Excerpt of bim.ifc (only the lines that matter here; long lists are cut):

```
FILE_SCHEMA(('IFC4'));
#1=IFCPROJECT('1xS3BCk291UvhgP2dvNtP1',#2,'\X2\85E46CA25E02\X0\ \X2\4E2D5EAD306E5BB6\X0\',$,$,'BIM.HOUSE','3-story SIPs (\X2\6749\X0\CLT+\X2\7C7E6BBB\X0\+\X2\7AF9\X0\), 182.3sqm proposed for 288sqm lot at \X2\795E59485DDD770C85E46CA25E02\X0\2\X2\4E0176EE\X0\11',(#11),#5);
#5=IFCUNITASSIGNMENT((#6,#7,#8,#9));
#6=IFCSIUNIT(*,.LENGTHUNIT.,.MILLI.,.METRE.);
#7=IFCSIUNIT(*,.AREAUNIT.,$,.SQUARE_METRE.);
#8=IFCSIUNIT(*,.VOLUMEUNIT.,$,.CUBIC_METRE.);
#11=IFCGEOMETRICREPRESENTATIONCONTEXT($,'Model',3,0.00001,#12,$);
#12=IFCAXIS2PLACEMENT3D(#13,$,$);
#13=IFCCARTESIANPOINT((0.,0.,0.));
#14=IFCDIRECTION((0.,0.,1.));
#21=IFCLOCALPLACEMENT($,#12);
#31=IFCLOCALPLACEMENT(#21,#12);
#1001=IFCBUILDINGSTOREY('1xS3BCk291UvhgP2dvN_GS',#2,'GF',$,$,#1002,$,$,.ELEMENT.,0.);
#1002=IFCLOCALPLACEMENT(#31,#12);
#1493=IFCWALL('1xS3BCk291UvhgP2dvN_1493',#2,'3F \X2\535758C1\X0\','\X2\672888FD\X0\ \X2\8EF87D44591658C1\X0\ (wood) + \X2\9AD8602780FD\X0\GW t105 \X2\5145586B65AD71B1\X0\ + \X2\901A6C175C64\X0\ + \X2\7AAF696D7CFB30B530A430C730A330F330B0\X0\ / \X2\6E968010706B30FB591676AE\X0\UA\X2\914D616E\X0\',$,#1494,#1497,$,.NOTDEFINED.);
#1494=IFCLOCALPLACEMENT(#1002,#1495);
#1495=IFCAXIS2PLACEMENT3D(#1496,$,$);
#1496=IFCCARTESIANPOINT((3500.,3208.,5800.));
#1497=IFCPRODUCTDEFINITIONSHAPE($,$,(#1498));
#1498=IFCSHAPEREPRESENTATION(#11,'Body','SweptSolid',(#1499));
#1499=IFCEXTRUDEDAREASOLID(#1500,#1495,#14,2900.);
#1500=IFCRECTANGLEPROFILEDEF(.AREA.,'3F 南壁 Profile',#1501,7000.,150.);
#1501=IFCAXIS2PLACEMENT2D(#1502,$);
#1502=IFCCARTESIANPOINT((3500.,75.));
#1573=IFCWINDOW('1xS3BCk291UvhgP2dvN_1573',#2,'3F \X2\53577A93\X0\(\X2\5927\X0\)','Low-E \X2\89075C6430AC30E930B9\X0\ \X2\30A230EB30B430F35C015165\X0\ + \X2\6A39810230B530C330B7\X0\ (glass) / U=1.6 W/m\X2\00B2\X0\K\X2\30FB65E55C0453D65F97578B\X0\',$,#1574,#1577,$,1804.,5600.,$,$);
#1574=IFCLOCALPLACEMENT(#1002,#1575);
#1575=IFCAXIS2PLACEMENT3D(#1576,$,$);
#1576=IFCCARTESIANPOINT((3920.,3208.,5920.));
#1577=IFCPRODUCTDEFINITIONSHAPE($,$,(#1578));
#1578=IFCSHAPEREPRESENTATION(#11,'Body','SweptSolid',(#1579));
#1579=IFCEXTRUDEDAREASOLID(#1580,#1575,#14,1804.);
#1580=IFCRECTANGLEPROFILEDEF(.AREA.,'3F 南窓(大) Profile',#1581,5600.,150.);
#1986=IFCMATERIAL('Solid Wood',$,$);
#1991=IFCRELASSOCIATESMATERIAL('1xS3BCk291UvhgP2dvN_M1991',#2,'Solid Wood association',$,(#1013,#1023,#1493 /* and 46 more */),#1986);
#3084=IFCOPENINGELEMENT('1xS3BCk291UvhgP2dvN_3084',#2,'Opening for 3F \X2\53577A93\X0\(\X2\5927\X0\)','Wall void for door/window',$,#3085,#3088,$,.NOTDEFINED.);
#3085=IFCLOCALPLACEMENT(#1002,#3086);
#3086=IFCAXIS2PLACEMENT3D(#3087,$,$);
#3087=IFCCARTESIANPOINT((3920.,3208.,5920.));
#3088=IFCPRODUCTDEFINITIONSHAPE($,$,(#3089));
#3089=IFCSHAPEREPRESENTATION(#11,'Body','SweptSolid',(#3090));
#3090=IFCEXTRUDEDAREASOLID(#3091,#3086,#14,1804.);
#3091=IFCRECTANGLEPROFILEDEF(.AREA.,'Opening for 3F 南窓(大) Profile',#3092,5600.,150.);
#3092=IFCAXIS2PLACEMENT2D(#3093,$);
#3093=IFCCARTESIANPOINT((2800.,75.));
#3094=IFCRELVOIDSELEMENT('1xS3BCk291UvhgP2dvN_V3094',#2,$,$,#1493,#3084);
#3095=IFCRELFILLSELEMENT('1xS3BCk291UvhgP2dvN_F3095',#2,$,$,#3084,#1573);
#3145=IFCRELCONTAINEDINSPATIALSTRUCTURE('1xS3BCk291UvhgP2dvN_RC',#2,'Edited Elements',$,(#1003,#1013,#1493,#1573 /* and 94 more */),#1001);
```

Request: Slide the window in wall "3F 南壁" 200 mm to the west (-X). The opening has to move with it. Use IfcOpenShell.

```python
import ifcopenshell
import ifcopenshell.api.geometry
import ifcopenshell.util.placement

model = ifcopenshell.open("bim.ifc")

window = model.by_guid("1xS3BCk291UvhgP2dvN_1573")
opening = window.FillsVoids[0].RelatingOpeningElement
wall = opening.VoidsElements[0].RelatingBuildingElement

wall_matrix = ifcopenshell.util.placement.get_local_placement(wall.ObjectPlacement)
shift = wall_matrix[:3, 0] * -200.0
before = ifcopenshell.util.placement.get_local_placement(window.ObjectPlacement)[:3, 3].copy()

# The window is not placed relative to its opening, so move both.
for product in (opening, window):
    matrix = ifcopenshell.util.placement.get_local_placement(product.ObjectPlacement)
    matrix[:3, 3] += shift
    ifcopenshell.api.geometry.edit_object_placement(model, product=product, matrix=matrix, is_si=False)

after = ifcopenshell.util.placement.get_local_placement(window.ObjectPlacement)[:3, 3]
print("window moved by", (after - before).round(3) + 0.0)

model.write("bim_edited.ifc")
```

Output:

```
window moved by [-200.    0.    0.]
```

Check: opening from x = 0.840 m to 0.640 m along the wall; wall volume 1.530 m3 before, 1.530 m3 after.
